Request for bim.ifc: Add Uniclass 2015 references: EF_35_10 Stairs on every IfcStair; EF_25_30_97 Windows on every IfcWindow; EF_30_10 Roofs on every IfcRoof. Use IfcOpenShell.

First a look at what the model holds.

```python
import ifcopenshell

model = ifcopenshell.open("bim.ifc")
print(model.schema)
print("classifications:", [c.Name for c in model.by_type("IfcClassification")])
for ifc_class in ("IfcDoor", "IfcRoof", "IfcStair", "IfcWall", "IfcWindow"):
    print(ifc_class, len(model.by_type(ifc_class)))
```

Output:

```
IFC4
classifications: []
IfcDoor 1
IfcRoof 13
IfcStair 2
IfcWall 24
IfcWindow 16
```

```python
import ifcopenshell
import ifcopenshell.api.classification

model = ifcopenshell.open("bim.ifc")

system = ifcopenshell.api.classification.add_classification(model, classification="Uniclass 2015")

codes = {
    "IfcStair": ("EF_35_10", "Stairs"),
    "IfcWindow": ("EF_25_30_97", "Windows"),
    "IfcRoof": ("EF_30_10", "Roofs"),
}
for ifc_class, (code, name) in codes.items():
    products = model.by_type(ifc_class)
    ifcopenshell.api.classification.add_reference(
        model, products=products, classification=system, identification=code, name=name
    )
    print(code, len(products))

model.write("bim-out.ifc")
```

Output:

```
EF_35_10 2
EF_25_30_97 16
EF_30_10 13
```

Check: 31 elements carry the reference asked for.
